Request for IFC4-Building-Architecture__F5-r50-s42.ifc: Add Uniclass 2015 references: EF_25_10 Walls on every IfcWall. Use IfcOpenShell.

First a look at what the model holds.

```python
import ifcopenshell

model = ifcopenshell.open("IFC4-Building-Architecture__F5-r50-s42.ifc")
print(model.schema)
print("classifications:", [c.Name for c in model.by_type("IfcClassification")])
for ifc_class in ("IfcDoor", "IfcRoof", "IfcStair", "IfcWall", "IfcWindow"):
    print(ifc_class, len(model.by_type(ifc_class)))
```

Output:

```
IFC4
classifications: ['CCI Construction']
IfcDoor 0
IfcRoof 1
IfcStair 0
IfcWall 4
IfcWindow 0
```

```python
import ifcopenshell
import ifcopenshell.api.classification

model = ifcopenshell.open("IFC4-Building-Architecture__F5-r50-s42.ifc")

system = ifcopenshell.api.classification.add_classification(model, classification="Uniclass 2015")

codes = {
    "IfcWall": ("EF_25_10", "Walls"),
}
for ifc_class, (code, name) in codes.items():
    products = model.by_type(ifc_class)
    ifcopenshell.api.classification.add_reference(
        model, products=products, classification=system, identification=code, name=name
    )
    print(code, len(products))

model.write("IFC4-Building-Architecture__F5-r50-s42_edited.ifc")
```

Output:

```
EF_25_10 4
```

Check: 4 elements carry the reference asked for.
